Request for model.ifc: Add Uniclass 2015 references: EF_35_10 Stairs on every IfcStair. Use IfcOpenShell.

First a look at what the model holds.

```python
import ifcopenshell

model = ifcopenshell.open("model.ifc")
print(model.schema)
print("classifications:", [c.Name for c in model.by_type("IfcClassification")])
for ifc_class in ("IfcDoor", "IfcRoof", "IfcStair", "IfcWall", "IfcWindow"):
    print(ifc_class, len(model.by_type(ifc_class)))
```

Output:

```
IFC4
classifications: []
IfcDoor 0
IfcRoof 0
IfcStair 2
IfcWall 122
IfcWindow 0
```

```python
import ifcopenshell
import ifcopenshell.api.classification

model = ifcopenshell.open("model.ifc")

system = ifcopenshell.api.classification.add_classification(model, classification="Uniclass 2015")

codes = {
    "IfcStair": ("EF_35_10", "Stairs"),
}
for ifc_class, (code, name) in codes.items():
    products = model.by_type(ifc_class)
    ifcopenshell.api.classification.add_reference(
        model, products=products, classification=system, identification=code, name=name
    )
    print(code, len(products))

model.write("model_edited.ifc")
```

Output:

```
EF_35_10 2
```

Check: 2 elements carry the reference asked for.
